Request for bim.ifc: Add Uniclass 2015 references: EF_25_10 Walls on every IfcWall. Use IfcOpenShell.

First a look at what the model holds.

```python
import ifcopenshell

model = ifcopenshell.open("bim.ifc")
print(model.schema)
print("classifications:", [c.Name for c in model.by_type("IfcClassification")])
for ifc_class in ("IfcDoor", "IfcRoof", "IfcStair", "IfcWall", "IfcWindow"):
    print(ifc_class, len(model.by_type(ifc_class)))
```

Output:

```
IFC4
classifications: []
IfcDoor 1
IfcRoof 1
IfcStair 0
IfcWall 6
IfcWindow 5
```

```python
import ifcopenshell
import ifcopenshell.api.classification

model = ifcopenshell.open("bim.ifc")

system = ifcopenshell.api.classification.add_classification(model, classification="Uniclass 2015")

codes = {
    "IfcWall": ("EF_25_10", "Walls"),
}
for ifc_class, (code, name) in codes.items():
    products = model.by_type(ifc_class)
    ifcopenshell.api.classification.add_reference(
        model, products=products, classification=system, identification=code, name=name
    )
    print(code, len(products))

model.write("bim_edited.ifc")
```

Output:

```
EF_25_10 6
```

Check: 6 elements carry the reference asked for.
